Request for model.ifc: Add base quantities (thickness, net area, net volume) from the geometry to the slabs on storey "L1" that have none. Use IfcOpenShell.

First a look at what the model holds.

```python
import ifcopenshell
import ifcopenshell.util.element
import ifcopenshell.util.unit

model = ifcopenshell.open("model.ifc")
print(model.schema)
for unit_type in ("LENGTHUNIT", "AREAUNIT", "VOLUMEUNIT"):
    print(unit_type, ifcopenshell.util.unit.calculate_unit_scale(model, unit_type))
storey = next(s for s in model.by_type("IfcBuildingStorey") if s.Name == "L1")
slabs = [e for e in ifcopenshell.util.element.get_decomposition(storey) if e.is_a("IfcSlab")]
for e in sorted(slabs, key=lambda e: e.id()):
    print(e.id(), e.is_a(), e.Name, list(ifcopenshell.util.element.get_psets(e, qtos_only=True)), sep=" | ")
```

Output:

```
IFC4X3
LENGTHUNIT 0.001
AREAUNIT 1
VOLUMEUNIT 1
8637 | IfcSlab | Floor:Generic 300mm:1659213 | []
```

```python
import ifcopenshell
import ifcopenshell.api.pset
import ifcopenshell.geom
import ifcopenshell.util.element
import ifcopenshell.util.shape
import ifcopenshell.util.unit

model = ifcopenshell.open("model.ifc")
unit_scale = ifcopenshell.util.unit.calculate_unit_scale(model)
area_scale = ifcopenshell.util.unit.calculate_unit_scale(model, "AREAUNIT")
volume_scale = ifcopenshell.util.unit.calculate_unit_scale(model, "VOLUMEUNIT")
settings = ifcopenshell.geom.settings()

storey = next(s for s in model.by_type("IfcBuildingStorey") if s.Name == "L1")
slabs = [e for e in ifcopenshell.util.element.get_decomposition(storey) if e.is_a("IfcSlab")]

for e in sorted(slabs, key=lambda e: e.id()):
    if ifcopenshell.util.element.get_psets(e, qtos_only=True, should_inherit=False):
        continue
    # Geometry comes back in metres, in the element's own axes.
    shape = ifcopenshell.geom.create_shape(settings, e)
    values = {
        "Width": ifcopenshell.util.shape.get_z(shape.geometry) / unit_scale,
        "NetArea": ifcopenshell.util.shape.get_footprint_area(shape.geometry) / area_scale,
        "NetVolume": ifcopenshell.util.shape.get_volume(shape.geometry) / volume_scale,
    }
    qto = ifcopenshell.api.pset.add_qto(model, product=e, name="Qto_SlabBaseQuantities")
    ifcopenshell.api.pset.edit_qto(model, qto=qto, properties=values)
    print(e.id(), {k: round(v, 3) for k, v in values.items()})

model.write("model_v2.ifc")
```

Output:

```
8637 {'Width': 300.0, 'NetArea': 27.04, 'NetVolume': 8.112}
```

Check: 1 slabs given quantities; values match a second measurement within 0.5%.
